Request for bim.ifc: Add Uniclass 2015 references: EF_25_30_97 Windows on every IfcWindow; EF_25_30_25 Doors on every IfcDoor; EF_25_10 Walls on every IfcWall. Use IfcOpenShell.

First a look at what the model holds.

```python
import ifcopenshell

model = ifcopenshell.open("bim.ifc")
print(model.schema)
print("classifications:", [c.Name for c in model.by_type("IfcClassification")])
for ifc_class in ("IfcDoor", "IfcRoof", "IfcStair", "IfcWall", "IfcWindow"):
    print(ifc_class, len(model.by_type(ifc_class)))
```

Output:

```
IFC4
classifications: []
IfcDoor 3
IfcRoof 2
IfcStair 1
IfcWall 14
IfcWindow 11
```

```python
import ifcopenshell
import ifcopenshell.api.classification

model = ifcopenshell.open("bim.ifc")

system = ifcopenshell.api.classification.add_classification(model, classification="Uniclass 2015")

codes = {
    "IfcWindow": ("EF_25_30_97", "Windows"),
    "IfcDoor": ("EF_25_30_25", "Doors"),
    "IfcWall": ("EF_25_10", "Walls"),
}
for ifc_class, (code, name) in codes.items():
    products = model.by_type(ifc_class)
    ifcopenshell.api.classification.add_reference(
        model, products=products, classification=system, identification=code, name=name
    )
    print(code, len(products))

model.write("bim-out.ifc")
```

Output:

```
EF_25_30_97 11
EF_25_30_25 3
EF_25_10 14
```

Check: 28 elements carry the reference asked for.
